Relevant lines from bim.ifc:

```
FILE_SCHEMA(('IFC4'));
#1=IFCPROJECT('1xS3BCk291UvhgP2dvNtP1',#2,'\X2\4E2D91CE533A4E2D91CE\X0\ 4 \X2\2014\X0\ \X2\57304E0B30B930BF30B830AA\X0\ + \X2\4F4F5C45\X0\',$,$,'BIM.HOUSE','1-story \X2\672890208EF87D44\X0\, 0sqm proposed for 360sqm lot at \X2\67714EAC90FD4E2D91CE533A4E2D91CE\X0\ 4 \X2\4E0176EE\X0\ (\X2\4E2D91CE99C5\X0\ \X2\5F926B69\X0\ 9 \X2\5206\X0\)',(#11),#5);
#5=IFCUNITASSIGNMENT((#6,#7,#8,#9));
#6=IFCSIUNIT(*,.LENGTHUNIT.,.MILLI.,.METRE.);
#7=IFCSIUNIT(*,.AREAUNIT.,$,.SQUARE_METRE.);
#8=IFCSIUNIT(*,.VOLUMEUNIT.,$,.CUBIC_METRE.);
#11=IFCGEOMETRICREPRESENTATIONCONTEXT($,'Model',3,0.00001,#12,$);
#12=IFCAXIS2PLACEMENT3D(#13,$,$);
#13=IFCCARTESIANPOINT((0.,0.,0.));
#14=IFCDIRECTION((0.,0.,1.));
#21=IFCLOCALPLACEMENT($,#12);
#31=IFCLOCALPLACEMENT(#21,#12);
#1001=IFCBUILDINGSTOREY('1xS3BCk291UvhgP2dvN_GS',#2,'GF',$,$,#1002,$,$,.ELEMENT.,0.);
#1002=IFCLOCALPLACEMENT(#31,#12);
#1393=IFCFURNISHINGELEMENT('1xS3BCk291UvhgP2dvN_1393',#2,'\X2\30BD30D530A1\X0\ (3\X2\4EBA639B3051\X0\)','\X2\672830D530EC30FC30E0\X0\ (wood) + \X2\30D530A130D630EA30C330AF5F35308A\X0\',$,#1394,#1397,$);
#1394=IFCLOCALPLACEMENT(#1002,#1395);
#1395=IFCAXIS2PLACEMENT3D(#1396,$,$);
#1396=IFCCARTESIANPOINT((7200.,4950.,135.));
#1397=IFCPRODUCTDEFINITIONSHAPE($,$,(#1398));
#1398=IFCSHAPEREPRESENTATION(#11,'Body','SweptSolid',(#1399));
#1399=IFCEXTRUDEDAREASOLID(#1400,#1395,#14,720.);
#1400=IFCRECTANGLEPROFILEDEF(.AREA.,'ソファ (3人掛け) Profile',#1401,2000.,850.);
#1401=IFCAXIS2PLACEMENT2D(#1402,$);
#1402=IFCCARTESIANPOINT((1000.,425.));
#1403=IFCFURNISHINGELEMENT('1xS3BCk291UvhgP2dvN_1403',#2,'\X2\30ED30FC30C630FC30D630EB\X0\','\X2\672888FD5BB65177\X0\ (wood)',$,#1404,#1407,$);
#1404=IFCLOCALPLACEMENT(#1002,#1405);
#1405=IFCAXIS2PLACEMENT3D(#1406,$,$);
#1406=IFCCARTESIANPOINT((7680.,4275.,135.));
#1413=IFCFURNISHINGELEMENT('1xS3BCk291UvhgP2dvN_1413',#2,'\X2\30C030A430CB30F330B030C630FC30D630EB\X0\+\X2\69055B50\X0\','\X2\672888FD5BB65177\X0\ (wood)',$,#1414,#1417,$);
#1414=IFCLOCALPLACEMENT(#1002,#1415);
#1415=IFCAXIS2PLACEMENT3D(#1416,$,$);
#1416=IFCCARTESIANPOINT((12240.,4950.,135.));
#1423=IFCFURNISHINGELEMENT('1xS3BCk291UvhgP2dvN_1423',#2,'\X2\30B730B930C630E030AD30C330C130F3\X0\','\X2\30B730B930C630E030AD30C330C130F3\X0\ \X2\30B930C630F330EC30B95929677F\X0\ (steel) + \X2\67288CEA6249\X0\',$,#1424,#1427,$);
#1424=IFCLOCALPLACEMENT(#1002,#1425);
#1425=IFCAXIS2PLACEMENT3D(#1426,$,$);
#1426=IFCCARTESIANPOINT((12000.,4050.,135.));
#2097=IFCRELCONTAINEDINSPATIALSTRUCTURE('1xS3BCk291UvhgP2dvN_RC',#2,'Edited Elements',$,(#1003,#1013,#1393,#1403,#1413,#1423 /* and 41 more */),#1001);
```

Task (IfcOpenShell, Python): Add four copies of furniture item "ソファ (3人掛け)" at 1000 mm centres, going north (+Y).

```python
import numpy as np
import ifcopenshell
import ifcopenshell.api.geometry
import ifcopenshell.api.root
import ifcopenshell.util.element
import ifcopenshell.util.placement
import ifcopenshell.util.unit

model = ifcopenshell.open("bim.ifc")
unit_scale = ifcopenshell.util.unit.calculate_unit_scale(model)


def reuse_history(source, copy):
    """copy_class also copies each property set's owner history, people and application; keep the originals."""
    for rel in copy.IsDefinedBy:
        if rel.is_a("IfcRelDefinesByProperties") and (history := rel.RelatingPropertyDefinition.OwnerHistory):
            rel.RelatingPropertyDefinition.OwnerHistory = source.OwnerHistory
            ifcopenshell.util.element.remove_deep2(model, history)


source = model.by_guid("1xS3BCk291UvhgP2dvN_1393")
base = ifcopenshell.util.placement.get_local_placement(source.ObjectPlacement)
step = np.array([0.0, 1.0, 0.0]) * 1 / unit_scale

for i in range(1, 5):
    copy = ifcopenshell.api.root.copy_class(model, product=source)
    copy.Representation = ifcopenshell.util.element.copy_deep(
        model, source.Representation, exclude=["IfcGeometricRepresentationContext", "IfcRepresentationMap"]
    )
    reuse_history(source, copy)
    matrix = base.copy()
    matrix[:3, 3] += i * step
    print("added at", matrix[:3, 3].round(3) + 0.0)
    ifcopenshell.api.geometry.edit_object_placement(model, product=copy, matrix=matrix, is_si=False)

model.write("bim_updated.ifc")
```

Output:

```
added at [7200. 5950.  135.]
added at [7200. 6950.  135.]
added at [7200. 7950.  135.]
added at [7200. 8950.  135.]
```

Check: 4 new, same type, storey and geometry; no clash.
